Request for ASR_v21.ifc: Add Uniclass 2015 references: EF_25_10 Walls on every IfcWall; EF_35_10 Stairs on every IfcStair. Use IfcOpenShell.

First a look at what the model holds.

```python
import ifcopenshell

model = ifcopenshell.open("ASR_v21.ifc")
print(model.schema)
print("classifications:", [c.Name for c in model.by_type("IfcClassification")])
for ifc_class in ("IfcDoor", "IfcRoof", "IfcStair", "IfcWall", "IfcWindow"):
    print(ifc_class, len(model.by_type(ifc_class)))
```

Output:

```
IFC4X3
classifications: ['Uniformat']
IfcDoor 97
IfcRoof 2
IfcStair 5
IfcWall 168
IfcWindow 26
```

```python
import ifcopenshell
import ifcopenshell.api.classification

model = ifcopenshell.open("ASR_v21.ifc")

system = ifcopenshell.api.classification.add_classification(model, classification="Uniclass 2015")

codes = {
    "IfcWall": ("EF_25_10", "Walls"),
    "IfcStair": ("EF_35_10", "Stairs"),
}
for ifc_class, (code, name) in codes.items():
    products = model.by_type(ifc_class)
    ifcopenshell.api.classification.add_reference(
        model, products=products, classification=system, identification=code, name=name
    )
    print(code, len(products))

model.write("ASR_v21_updated.ifc")
```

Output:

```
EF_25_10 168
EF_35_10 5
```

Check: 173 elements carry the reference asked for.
